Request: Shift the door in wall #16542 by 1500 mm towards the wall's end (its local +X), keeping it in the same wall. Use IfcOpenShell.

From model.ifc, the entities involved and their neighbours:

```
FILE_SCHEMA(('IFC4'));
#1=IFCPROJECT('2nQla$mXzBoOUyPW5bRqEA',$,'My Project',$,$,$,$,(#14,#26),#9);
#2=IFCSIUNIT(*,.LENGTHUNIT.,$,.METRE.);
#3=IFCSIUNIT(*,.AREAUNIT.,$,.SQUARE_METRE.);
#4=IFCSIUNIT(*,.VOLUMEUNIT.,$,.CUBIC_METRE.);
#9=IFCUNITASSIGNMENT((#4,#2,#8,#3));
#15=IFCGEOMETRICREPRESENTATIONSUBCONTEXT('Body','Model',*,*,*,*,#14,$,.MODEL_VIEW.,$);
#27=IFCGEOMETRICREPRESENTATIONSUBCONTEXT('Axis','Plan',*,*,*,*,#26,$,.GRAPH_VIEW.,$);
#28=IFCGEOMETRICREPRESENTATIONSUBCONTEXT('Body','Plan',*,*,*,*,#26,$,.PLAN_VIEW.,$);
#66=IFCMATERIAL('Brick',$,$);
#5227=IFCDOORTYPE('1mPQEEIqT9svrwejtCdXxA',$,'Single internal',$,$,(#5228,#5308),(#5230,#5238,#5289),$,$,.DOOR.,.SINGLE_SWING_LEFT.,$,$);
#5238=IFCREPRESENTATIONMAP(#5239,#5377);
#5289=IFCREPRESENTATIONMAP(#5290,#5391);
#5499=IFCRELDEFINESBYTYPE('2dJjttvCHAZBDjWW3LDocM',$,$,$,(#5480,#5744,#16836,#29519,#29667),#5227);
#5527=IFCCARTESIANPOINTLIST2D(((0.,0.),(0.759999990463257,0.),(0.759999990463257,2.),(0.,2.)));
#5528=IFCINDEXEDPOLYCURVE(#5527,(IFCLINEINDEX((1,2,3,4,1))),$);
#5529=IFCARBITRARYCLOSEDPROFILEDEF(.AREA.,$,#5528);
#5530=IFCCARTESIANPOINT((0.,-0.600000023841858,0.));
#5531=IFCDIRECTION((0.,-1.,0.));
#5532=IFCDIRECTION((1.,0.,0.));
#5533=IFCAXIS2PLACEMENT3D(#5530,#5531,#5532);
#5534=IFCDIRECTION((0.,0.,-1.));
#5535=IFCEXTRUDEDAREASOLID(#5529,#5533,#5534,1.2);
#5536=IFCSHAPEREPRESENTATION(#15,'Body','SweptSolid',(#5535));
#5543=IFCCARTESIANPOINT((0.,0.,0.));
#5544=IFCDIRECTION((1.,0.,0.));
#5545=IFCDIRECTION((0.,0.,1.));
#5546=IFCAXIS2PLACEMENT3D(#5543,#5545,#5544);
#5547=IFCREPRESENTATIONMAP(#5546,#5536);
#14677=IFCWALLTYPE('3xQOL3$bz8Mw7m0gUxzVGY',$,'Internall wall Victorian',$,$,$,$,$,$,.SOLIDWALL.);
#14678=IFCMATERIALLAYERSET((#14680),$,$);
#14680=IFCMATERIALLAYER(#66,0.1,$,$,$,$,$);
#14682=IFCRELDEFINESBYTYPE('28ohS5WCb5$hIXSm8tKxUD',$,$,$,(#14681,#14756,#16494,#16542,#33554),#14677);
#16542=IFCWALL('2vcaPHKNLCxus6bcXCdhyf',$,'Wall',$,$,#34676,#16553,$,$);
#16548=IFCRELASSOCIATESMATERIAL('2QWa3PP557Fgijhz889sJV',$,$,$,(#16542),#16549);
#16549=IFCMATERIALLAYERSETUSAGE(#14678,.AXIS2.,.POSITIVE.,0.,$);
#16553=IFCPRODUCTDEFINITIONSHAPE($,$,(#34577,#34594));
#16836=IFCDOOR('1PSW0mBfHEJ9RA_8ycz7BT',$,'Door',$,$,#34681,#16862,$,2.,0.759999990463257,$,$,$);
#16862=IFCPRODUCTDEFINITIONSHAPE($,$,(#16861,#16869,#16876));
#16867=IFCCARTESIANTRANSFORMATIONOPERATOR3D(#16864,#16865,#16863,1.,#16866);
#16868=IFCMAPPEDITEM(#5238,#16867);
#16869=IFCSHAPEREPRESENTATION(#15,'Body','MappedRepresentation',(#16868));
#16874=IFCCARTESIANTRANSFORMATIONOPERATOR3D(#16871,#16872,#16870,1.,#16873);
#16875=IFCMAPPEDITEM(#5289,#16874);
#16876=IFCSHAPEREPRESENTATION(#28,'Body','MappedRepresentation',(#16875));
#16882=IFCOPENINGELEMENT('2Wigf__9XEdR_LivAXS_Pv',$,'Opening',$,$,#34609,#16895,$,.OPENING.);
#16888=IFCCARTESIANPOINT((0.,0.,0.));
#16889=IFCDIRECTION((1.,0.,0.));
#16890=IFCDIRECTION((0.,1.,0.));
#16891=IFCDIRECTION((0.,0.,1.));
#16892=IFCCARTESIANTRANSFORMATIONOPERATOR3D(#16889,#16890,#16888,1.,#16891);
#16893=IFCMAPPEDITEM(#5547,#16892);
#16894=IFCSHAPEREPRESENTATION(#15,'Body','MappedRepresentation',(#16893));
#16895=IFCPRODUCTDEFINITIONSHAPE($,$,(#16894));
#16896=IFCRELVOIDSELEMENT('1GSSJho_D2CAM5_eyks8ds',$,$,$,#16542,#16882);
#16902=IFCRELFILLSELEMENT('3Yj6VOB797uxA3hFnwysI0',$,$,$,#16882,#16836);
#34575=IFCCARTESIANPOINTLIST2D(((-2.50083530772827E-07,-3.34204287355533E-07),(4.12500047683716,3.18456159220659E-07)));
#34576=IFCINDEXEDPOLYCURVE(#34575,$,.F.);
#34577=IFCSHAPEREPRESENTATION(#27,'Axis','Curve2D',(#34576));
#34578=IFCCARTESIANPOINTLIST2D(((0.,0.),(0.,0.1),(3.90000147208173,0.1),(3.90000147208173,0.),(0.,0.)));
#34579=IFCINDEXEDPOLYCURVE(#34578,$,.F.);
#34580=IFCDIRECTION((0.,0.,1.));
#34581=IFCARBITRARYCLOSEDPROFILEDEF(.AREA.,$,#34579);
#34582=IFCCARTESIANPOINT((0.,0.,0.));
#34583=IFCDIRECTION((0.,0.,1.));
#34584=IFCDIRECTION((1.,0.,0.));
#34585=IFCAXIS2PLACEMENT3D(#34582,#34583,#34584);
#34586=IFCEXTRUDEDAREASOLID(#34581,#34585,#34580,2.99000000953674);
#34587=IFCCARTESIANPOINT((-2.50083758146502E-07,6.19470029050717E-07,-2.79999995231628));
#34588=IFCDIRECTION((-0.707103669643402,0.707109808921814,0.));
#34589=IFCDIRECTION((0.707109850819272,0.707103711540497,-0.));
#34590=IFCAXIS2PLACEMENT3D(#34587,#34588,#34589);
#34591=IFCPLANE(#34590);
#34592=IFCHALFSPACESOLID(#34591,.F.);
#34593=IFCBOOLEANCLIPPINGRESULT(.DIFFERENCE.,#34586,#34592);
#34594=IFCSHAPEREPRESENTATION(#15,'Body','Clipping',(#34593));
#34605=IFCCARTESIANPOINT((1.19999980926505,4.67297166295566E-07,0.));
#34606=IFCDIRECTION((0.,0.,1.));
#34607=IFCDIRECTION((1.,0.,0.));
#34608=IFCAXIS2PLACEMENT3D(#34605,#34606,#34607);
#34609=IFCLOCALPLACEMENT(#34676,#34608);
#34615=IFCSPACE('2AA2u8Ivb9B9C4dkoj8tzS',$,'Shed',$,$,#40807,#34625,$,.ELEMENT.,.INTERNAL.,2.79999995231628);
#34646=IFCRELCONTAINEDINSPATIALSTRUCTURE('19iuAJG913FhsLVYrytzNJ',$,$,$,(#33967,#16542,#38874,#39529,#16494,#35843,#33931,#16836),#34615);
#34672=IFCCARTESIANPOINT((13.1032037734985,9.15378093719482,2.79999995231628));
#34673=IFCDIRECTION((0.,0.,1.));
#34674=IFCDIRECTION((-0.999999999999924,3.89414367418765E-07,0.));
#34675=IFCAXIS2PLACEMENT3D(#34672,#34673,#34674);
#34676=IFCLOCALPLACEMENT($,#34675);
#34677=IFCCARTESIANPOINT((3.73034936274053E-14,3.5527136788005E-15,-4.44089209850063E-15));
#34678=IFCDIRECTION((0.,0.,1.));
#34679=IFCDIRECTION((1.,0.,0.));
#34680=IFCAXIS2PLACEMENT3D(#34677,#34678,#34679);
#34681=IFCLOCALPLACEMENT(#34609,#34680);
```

```python
import ifcopenshell
import ifcopenshell.api.geometry
import ifcopenshell.util.placement

model = ifcopenshell.open("model.ifc")

door = model.by_guid("1PSW0mBfHEJ9RA_8ycz7BT")
opening = door.FillsVoids[0].RelatingOpeningElement
wall = opening.VoidsElements[0].RelatingBuildingElement

wall_matrix = ifcopenshell.util.placement.get_local_placement(wall.ObjectPlacement)
shift = wall_matrix[:3, 0] * 1.5
before = ifcopenshell.util.placement.get_local_placement(door.ObjectPlacement)[:3, 3].copy()

# The door is placed relative to its opening, so it follows when the opening moves.
matrix = ifcopenshell.util.placement.get_local_placement(opening.ObjectPlacement)
matrix[:3, 3] += shift
ifcopenshell.api.geometry.edit_object_placement(
    model, product=opening, matrix=matrix, is_si=False, should_transform_children=True
)

after = ifcopenshell.util.placement.get_local_placement(door.ObjectPlacement)[:3, 3]
print("door moved by", (after - before).round(3) + 0.0)

model.write("model_edited.ifc")
```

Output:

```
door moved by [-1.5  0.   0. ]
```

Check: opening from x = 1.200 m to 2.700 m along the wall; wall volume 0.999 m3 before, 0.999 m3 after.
